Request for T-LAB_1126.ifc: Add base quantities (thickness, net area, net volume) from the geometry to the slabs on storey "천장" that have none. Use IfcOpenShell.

First a look at what the model holds.

```python
import ifcopenshell
import ifcopenshell.util.element
import ifcopenshell.util.unit

model = ifcopenshell.open("T-LAB_1126.ifc")
print(model.schema)
for unit_type in ("LENGTHUNIT", "AREAUNIT", "VOLUMEUNIT"):
    print(unit_type, ifcopenshell.util.unit.calculate_unit_scale(model, unit_type))
storey = next(s for s in model.by_type("IfcBuildingStorey") if s.Name == "천장")
slabs = [e for e in ifcopenshell.util.element.get_decomposition(storey) if e.is_a("IfcSlab")]
for e in sorted(slabs, key=lambda e: e.id()):
    print(e.id(), e.is_a(), e.Name, list(ifcopenshell.util.element.get_psets(e, qtos_only=True)), sep=" | ")
```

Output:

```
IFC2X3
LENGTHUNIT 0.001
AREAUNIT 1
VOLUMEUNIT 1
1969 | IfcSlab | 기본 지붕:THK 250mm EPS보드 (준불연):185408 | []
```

```python
import ifcopenshell
import ifcopenshell.api.pset
import ifcopenshell.geom
import ifcopenshell.util.element
import ifcopenshell.util.shape
import ifcopenshell.util.unit

model = ifcopenshell.open("T-LAB_1126.ifc")
unit_scale = ifcopenshell.util.unit.calculate_unit_scale(model)
area_scale = ifcopenshell.util.unit.calculate_unit_scale(model, "AREAUNIT")
volume_scale = ifcopenshell.util.unit.calculate_unit_scale(model, "VOLUMEUNIT")
settings = ifcopenshell.geom.settings()

storey = next(s for s in model.by_type("IfcBuildingStorey") if s.Name == "천장")
slabs = [e for e in ifcopenshell.util.element.get_decomposition(storey) if e.is_a("IfcSlab")]

for e in sorted(slabs, key=lambda e: e.id()):
    if ifcopenshell.util.element.get_psets(e, qtos_only=True, should_inherit=False):
        continue
    # Geometry comes back in metres, in the element's own axes.
    shape = ifcopenshell.geom.create_shape(settings, e)
    values = {
        "Width": ifcopenshell.util.shape.get_z(shape.geometry) / unit_scale,
        "NetArea": ifcopenshell.util.shape.get_footprint_area(shape.geometry) / area_scale,
        "NetVolume": ifcopenshell.util.shape.get_volume(shape.geometry) / volume_scale,
    }
    qto = ifcopenshell.api.pset.add_qto(model, product=e, name="BaseQuantities")
    ifcopenshell.api.pset.edit_qto(model, qto=qto, properties=values)
    print(e.id(), {k: round(v, 3) for k, v in values.items()})

model.write("T-LAB_1126_edited.ifc")
```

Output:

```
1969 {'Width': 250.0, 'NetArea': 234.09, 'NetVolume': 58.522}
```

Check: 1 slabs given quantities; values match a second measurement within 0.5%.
